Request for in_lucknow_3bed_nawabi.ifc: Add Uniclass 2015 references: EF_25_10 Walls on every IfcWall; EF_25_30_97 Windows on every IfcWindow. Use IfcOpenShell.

First a look at what the model holds.

```python
import ifcopenshell

model = ifcopenshell.open("in_lucknow_3bed_nawabi.ifc")
print(model.schema)
print("classifications:", [c.Name for c in model.by_type("IfcClassification")])
for ifc_class in ("IfcDoor", "IfcRoof", "IfcStair", "IfcWall", "IfcWindow"):
    print(ifc_class, len(model.by_type(ifc_class)))
```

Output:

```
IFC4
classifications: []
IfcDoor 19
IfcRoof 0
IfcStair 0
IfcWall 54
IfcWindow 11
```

```python
import ifcopenshell
import ifcopenshell.api.classification

model = ifcopenshell.open("in_lucknow_3bed_nawabi.ifc")

system = ifcopenshell.api.classification.add_classification(model, classification="Uniclass 2015")

codes = {
    "IfcWall": ("EF_25_10", "Walls"),
    "IfcWindow": ("EF_25_30_97", "Windows"),
}
for ifc_class, (code, name) in codes.items():
    products = model.by_type(ifc_class)
    ifcopenshell.api.classification.add_reference(
        model, products=products, classification=system, identification=code, name=name
    )
    print(code, len(products))

model.write("in_lucknow_3bed_nawabi_v2.ifc")
```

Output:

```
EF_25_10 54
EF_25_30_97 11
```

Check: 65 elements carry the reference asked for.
